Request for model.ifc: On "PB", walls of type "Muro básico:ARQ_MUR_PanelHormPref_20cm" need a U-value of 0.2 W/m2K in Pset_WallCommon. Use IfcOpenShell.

First a look at what the model holds.

```python
import ifcopenshell
import ifcopenshell.util.element

model = ifcopenshell.open("model.ifc")
print(model.schema)
storey = next(s for s in model.by_type("IfcBuildingStorey") if s.Name == "PB")
walls = [e for e in ifcopenshell.util.element.get_decomposition(storey) if e.is_a("IfcWall")]
seen = {}
for e in walls:
    element_type = ifcopenshell.util.element.get_type(e)
    key = (element_type.Name if element_type != e and element_type else None, ifcopenshell.util.element.get_pset(e, "Pset_WallCommon", "ThermalTransmittance"))
    seen[key] = seen.get(key, 0) + 1
for (name, value), count in sorted(seen.items(), key=str):
    print(count, "x", name, "|", value)
```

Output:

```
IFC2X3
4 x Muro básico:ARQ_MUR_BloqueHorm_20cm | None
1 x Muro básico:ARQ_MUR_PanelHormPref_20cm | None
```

```python
import ifcopenshell
import ifcopenshell.api.pset
import ifcopenshell.util.element

model = ifcopenshell.open("model.ifc")

storey = next(s for s in model.by_type("IfcBuildingStorey") if s.Name == "PB")
walls = [e for e in ifcopenshell.util.element.get_decomposition(storey) if e.is_a("IfcWall")]

count = 0
for e in walls:
    element_type = ifcopenshell.util.element.get_type(e)
    if element_type in (None, e) or element_type.Name != "Muro básico:ARQ_MUR_PanelHormPref_20cm":
        continue
    # add_pset returns the element's existing set when there is one.
    pset = ifcopenshell.api.pset.add_pset(model, product=e, name="Pset_WallCommon")
    ifcopenshell.api.pset.edit_pset(model, pset=pset, properties={"ThermalTransmittance": 0.2})
    count += 1

print(count, "walls updated")

model.write("model_v2.ifc")
```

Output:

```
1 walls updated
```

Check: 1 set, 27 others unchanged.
